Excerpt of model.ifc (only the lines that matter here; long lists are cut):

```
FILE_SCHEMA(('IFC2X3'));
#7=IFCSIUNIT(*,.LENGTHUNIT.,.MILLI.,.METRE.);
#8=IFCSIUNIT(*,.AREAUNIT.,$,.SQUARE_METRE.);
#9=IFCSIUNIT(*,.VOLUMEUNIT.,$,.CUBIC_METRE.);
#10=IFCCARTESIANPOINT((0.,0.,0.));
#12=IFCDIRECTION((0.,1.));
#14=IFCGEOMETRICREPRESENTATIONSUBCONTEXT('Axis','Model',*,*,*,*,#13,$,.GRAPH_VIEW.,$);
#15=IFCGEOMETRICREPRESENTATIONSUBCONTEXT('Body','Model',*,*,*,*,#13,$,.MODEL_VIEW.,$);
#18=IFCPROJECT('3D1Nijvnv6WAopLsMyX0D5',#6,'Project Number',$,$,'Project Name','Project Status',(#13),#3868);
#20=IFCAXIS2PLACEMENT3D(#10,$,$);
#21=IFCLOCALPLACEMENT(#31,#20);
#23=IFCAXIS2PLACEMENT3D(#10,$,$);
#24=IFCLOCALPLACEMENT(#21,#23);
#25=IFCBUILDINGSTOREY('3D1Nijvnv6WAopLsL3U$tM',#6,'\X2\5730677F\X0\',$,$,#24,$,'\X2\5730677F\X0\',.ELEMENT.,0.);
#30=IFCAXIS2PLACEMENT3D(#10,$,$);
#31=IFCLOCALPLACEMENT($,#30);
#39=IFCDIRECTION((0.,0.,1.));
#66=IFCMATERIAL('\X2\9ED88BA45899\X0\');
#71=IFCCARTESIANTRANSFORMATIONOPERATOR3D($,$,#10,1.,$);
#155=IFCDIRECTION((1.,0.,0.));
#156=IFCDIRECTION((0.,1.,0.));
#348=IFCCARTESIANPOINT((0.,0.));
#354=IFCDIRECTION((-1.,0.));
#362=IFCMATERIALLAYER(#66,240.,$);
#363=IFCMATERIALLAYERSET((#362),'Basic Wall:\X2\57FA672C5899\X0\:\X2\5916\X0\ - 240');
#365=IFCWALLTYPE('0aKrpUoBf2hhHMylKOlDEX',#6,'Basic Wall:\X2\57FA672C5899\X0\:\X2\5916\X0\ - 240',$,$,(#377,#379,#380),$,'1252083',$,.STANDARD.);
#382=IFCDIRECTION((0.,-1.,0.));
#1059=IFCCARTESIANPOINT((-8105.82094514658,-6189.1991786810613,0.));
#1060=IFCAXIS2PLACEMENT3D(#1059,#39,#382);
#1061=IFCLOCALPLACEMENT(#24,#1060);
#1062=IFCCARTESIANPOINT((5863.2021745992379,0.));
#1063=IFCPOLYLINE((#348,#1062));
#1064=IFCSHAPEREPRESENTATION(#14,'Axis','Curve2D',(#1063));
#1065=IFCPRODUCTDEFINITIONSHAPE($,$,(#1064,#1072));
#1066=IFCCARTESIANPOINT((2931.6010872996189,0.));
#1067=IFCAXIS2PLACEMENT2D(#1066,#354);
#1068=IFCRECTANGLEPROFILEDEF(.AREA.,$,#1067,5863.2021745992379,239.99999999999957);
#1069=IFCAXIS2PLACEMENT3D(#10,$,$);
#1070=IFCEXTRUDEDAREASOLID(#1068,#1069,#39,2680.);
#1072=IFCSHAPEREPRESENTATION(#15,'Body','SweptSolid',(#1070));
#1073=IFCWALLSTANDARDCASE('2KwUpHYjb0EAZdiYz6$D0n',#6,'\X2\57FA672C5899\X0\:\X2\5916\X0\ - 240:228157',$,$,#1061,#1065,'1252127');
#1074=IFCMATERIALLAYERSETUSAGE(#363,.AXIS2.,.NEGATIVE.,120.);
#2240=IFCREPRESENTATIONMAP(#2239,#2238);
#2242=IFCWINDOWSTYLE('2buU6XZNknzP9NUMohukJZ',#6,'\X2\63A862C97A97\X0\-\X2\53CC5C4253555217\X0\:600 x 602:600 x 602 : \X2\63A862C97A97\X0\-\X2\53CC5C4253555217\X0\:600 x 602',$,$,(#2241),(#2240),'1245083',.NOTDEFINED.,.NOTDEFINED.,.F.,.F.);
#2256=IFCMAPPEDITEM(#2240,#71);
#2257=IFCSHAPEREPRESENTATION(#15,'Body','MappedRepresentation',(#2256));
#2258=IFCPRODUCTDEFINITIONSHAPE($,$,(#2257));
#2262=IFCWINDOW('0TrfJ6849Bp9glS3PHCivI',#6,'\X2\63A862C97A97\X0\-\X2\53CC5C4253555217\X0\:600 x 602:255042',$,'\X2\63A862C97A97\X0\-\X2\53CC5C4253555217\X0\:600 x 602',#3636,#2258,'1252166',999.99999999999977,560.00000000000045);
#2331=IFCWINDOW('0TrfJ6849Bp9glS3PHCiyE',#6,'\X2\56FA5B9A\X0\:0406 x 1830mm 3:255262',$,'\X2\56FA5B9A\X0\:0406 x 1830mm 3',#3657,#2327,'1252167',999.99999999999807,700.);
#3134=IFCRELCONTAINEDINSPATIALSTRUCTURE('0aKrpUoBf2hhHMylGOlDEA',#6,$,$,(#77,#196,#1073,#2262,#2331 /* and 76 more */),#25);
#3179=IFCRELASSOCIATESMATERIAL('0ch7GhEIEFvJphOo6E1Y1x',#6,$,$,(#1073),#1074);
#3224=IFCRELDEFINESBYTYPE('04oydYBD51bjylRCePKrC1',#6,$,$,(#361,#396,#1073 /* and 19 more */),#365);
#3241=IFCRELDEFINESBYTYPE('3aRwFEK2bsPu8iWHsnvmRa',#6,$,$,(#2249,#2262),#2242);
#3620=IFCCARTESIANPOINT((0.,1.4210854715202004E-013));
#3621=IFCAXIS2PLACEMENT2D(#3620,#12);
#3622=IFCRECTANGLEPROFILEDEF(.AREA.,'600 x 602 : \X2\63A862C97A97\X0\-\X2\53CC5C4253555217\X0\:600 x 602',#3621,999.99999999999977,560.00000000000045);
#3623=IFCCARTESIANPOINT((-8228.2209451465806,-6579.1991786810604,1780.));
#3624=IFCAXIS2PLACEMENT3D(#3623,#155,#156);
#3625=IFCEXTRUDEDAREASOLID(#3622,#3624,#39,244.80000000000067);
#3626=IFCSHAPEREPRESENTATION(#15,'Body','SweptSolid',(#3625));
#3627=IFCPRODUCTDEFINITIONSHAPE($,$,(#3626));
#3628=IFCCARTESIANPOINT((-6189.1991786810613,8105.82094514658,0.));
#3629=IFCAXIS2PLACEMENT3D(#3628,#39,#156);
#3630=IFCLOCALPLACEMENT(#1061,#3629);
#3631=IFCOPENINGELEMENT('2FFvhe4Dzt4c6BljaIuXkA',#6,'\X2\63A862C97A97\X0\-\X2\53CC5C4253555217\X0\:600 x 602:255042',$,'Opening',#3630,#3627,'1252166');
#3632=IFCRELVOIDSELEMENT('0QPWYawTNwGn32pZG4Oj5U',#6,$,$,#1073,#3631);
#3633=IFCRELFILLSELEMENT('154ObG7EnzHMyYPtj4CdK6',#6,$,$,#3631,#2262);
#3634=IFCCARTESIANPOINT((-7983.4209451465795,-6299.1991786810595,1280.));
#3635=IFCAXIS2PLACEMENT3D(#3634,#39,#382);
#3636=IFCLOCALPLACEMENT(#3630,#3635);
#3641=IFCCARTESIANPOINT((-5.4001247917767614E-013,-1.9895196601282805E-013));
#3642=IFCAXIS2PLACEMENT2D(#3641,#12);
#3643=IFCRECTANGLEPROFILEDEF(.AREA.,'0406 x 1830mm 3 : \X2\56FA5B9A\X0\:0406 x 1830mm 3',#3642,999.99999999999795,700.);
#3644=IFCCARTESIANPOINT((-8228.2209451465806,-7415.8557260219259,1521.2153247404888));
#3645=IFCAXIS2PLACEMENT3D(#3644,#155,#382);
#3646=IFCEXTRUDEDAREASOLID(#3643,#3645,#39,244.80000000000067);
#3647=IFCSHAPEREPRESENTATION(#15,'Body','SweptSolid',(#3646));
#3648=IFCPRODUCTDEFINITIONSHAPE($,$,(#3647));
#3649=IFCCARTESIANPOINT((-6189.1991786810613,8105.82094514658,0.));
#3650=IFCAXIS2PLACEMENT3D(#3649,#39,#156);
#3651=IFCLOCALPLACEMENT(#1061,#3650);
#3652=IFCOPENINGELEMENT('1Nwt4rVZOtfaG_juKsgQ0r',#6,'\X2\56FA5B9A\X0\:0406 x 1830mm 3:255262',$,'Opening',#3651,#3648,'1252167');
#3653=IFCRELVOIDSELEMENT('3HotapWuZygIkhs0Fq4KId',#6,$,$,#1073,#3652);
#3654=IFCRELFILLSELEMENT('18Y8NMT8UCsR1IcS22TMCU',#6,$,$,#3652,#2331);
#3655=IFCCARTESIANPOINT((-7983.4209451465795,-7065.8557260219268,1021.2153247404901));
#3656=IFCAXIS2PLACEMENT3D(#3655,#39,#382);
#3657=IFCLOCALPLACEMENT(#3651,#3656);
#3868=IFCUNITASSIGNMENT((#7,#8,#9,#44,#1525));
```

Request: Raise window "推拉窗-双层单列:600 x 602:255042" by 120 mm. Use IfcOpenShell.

```python
import numpy as np
import ifcopenshell
import ifcopenshell.api.geometry
import ifcopenshell.util.placement
import ifcopenshell.util.unit

model = ifcopenshell.open("model.ifc")
unit_scale = ifcopenshell.util.unit.calculate_unit_scale(model)

window = model.by_guid("0TrfJ6849Bp9glS3PHCivI")
opening = window.FillsVoids[0].RelatingOpeningElement
dz = 0.12 / unit_scale

shift = np.array([0.0, 0.0, dz])
# The window is placed relative to its opening, so it follows when the opening moves.
matrix = ifcopenshell.util.placement.get_local_placement(opening.ObjectPlacement)
matrix[:3, 3] += shift
ifcopenshell.api.geometry.edit_object_placement(
    model, product=opening, matrix=matrix, is_si=False, should_transform_children=True
)

print(f"moved by {dz * unit_scale:+.3f} m")

model.write("model_v2.ifc")
```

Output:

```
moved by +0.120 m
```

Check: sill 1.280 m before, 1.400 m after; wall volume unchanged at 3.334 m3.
